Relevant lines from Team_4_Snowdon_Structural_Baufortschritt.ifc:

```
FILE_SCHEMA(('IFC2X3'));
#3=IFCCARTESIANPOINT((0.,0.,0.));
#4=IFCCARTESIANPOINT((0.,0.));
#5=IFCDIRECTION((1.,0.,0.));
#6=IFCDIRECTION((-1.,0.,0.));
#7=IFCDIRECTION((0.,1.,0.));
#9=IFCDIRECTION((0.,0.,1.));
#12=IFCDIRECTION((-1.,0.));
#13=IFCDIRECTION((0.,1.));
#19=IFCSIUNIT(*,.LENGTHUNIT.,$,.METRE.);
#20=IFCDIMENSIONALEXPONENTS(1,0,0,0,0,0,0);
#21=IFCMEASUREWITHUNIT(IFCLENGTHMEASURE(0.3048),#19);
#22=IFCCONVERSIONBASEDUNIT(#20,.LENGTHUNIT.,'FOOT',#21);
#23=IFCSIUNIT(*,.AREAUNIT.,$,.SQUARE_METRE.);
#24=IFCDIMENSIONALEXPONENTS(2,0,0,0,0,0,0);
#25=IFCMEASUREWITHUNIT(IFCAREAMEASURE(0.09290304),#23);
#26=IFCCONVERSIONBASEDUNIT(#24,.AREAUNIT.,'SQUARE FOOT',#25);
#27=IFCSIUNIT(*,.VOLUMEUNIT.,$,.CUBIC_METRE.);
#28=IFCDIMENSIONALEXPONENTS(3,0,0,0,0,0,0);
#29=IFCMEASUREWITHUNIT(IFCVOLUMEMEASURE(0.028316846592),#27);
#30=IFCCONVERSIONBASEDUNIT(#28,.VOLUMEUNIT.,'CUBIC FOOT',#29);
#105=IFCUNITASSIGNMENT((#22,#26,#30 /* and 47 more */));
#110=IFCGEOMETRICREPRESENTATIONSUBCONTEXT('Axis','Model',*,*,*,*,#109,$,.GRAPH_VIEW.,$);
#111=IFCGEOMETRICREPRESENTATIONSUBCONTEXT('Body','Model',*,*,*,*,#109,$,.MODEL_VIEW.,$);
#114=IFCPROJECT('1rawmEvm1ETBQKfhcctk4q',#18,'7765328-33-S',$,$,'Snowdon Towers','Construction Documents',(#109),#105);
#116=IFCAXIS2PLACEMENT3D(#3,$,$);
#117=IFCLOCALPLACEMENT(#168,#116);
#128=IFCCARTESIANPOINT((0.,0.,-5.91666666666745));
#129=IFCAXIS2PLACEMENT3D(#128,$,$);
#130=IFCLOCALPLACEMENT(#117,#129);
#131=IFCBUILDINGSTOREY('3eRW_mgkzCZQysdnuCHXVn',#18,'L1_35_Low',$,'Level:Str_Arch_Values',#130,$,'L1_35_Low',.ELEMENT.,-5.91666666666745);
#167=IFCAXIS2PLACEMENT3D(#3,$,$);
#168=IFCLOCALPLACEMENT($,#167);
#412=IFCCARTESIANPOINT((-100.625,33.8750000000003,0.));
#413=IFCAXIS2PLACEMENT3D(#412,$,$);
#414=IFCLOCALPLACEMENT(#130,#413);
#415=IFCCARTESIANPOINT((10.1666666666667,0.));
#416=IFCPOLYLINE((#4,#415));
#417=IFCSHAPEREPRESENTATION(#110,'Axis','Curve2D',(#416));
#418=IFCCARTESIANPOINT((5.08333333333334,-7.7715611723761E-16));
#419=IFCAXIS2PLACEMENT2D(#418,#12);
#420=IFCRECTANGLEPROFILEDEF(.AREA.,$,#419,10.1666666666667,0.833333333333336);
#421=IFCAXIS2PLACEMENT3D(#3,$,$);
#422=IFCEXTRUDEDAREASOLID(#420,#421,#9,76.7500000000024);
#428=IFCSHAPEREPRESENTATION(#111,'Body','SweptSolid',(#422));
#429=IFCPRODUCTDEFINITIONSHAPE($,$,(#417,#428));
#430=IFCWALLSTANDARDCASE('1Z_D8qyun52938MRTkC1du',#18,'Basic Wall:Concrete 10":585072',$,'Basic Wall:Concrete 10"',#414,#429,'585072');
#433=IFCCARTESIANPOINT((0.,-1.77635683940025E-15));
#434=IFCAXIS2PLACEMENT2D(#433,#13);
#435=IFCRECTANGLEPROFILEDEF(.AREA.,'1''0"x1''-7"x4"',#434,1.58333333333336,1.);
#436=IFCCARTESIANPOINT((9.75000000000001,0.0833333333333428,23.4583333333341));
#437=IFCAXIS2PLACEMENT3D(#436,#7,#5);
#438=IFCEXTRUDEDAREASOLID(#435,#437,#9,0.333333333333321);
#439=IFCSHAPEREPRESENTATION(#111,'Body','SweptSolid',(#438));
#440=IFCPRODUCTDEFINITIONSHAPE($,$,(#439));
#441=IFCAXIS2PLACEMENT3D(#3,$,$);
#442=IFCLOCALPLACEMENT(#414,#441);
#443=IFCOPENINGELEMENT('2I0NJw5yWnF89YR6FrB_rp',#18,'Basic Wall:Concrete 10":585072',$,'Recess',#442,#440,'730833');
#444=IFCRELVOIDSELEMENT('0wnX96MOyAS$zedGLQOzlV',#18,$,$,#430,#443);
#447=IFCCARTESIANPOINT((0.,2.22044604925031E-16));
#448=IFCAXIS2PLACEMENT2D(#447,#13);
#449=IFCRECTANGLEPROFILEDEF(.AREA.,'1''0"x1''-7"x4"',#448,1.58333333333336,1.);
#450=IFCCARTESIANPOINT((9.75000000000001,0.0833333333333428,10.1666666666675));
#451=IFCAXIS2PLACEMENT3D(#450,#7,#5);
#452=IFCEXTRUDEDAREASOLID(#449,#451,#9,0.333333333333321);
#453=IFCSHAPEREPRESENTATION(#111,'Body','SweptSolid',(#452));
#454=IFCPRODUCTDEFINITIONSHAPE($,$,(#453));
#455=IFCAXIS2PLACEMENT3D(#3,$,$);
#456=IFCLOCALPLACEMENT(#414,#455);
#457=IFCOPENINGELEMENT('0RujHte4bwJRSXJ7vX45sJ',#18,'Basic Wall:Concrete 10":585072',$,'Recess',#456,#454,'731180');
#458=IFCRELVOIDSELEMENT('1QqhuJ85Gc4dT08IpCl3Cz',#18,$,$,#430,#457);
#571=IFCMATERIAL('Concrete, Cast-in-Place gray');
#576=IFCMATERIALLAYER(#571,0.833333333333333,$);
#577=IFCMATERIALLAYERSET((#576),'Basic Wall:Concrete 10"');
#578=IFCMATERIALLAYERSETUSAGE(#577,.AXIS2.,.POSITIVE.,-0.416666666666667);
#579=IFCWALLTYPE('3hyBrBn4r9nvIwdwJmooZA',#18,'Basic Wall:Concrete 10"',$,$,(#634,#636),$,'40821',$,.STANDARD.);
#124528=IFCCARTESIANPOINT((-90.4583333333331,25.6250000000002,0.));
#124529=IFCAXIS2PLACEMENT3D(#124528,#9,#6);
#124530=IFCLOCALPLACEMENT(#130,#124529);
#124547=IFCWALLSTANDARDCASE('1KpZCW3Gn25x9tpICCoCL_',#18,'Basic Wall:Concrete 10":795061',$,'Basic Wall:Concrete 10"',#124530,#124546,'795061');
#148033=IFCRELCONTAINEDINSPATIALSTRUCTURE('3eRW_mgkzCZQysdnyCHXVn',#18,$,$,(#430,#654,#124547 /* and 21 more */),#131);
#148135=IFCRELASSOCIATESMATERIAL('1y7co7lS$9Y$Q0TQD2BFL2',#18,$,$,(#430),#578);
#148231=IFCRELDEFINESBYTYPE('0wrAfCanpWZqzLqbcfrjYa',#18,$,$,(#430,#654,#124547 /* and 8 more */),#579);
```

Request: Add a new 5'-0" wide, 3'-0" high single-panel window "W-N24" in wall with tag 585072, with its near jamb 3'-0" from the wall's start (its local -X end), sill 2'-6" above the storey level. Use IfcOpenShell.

```python
import numpy as np
import ifcopenshell
import ifcopenshell.api.feature
import ifcopenshell.api.geometry
import ifcopenshell.api.root
import ifcopenshell.api.spatial
import ifcopenshell.api.type
import ifcopenshell.geom
import ifcopenshell.util.element
import ifcopenshell.util.placement
import ifcopenshell.util.representation
import ifcopenshell.util.shape
import ifcopenshell.util.unit

model = ifcopenshell.open("Team_4_Snowdon_Structural_Baufortschritt.ifc")
unit_scale = ifcopenshell.util.unit.calculate_unit_scale(model)
settings = ifcopenshell.geom.settings()


def volume(element):
    """Net volume in cubic metres, openings subtracted."""
    shape = ifcopenshell.geom.create_shape(settings, element)
    return ifcopenshell.util.shape.get_volume(shape.geometry)


wall = model.by_guid("1Z_D8qyun52938MRTkC1du")
storey = ifcopenshell.util.element.get_container(wall, ifc_class="IfcBuildingStorey")
context = ifcopenshell.util.representation.get_context(model, "Model", "Body", "MODEL_VIEW")
before = volume(wall)

width, height, from_end, sill = 1.524, 0.9144, 0.9144, 0.762  # metres

# The wall runs along its own X axis, and the end named is its -X end.
wall_shape = ifcopenshell.geom.create_shape(settings, wall)
x, y, z = ifcopenshell.util.shape.get_vertices(wall_shape.geometry).T
start = x.min() + from_end
face, thickness = float(y.min()), float(y.max() - y.min())
wall_matrix = ifcopenshell.util.placement.get_local_placement(wall.ObjectPlacement)
level = ifcopenshell.util.placement.get_local_placement(storey.ObjectPlacement)[2, 3]


def in_wall(x, y):
    """Placement at x, y metres in the wall's axes, at sill height."""
    matrix = wall_matrix.copy()
    matrix[:, 3] = wall_matrix @ np.array([x / unit_scale, y / unit_scale, 0.0, 1.0])
    matrix[2, 3] = level + sill / unit_scale
    return matrix


# Opening: a box that overshoots both wall faces by 50 mm.
opening = ifcopenshell.api.root.create_entity(model, ifc_class="IfcOpeningElement")
box = ifcopenshell.api.geometry.add_wall_representation(
    model, context=context, length=width, height=height, thickness=thickness + 0.1
)
ifcopenshell.api.geometry.assign_representation(model, product=opening, representation=box)
ifcopenshell.api.geometry.edit_object_placement(model, product=opening, matrix=in_wall(start, face - 0.05), is_si=False)
ifcopenshell.api.feature.add_feature(model, feature=opening, element=wall)

window = ifcopenshell.api.root.create_entity(model, ifc_class="IfcWindow", name="W-N24")
window.OverallWidth, window.OverallHeight = width / unit_scale, height / unit_scale
body = ifcopenshell.api.geometry.add_window_representation(
    model,
    context=context,
    overall_width=window.OverallWidth,
    overall_height=window.OverallHeight,
    partition_type="SINGLE_PANEL",
)
ifcopenshell.api.geometry.assign_representation(model, product=window, representation=body)
ifcopenshell.api.spatial.assign_container(model, products=[window], relating_structure=storey)
fills = ifcopenshell.api.feature.add_filling(model, opening=opening, element=window)
fills.OwnerHistory = window.OwnerHistory  # required in IFC2X3

# IFC2X3 keeps the operation on the window style.
style = ifcopenshell.api.root.create_entity(model, ifc_class="IfcWindowStyle", name="W-N24")
style.OperationType, style.ConstructionType = "SINGLE_PANEL", "NOTDEFINED"
style.ParameterTakesPrecedence = style.Sizeable = False
ifcopenshell.api.type.assign_type(model, related_objects=[window], relating_type=style)

# Centre the window in the wall's thickness.
ifcopenshell.api.geometry.edit_object_placement(model, product=window, matrix=in_wall(start, face), is_si=False)
window_shape = ifcopenshell.geom.create_shape(settings, window)
depth = ifcopenshell.util.shape.get_vertices(window_shape.geometry)[:, 1]
offset = face + thickness / 2 - (depth.min() + depth.max()) / 2
ifcopenshell.api.geometry.edit_object_placement(model, product=window, matrix=in_wall(start, offset), is_si=False)

after = volume(wall)

print(f"wall volume {before:.3f} -> {after:.3f} m3")

model.write("Team_4_Snowdon_Structural_Baufortschritt_v2.ifc")
```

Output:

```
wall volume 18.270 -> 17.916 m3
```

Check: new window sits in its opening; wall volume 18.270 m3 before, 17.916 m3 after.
